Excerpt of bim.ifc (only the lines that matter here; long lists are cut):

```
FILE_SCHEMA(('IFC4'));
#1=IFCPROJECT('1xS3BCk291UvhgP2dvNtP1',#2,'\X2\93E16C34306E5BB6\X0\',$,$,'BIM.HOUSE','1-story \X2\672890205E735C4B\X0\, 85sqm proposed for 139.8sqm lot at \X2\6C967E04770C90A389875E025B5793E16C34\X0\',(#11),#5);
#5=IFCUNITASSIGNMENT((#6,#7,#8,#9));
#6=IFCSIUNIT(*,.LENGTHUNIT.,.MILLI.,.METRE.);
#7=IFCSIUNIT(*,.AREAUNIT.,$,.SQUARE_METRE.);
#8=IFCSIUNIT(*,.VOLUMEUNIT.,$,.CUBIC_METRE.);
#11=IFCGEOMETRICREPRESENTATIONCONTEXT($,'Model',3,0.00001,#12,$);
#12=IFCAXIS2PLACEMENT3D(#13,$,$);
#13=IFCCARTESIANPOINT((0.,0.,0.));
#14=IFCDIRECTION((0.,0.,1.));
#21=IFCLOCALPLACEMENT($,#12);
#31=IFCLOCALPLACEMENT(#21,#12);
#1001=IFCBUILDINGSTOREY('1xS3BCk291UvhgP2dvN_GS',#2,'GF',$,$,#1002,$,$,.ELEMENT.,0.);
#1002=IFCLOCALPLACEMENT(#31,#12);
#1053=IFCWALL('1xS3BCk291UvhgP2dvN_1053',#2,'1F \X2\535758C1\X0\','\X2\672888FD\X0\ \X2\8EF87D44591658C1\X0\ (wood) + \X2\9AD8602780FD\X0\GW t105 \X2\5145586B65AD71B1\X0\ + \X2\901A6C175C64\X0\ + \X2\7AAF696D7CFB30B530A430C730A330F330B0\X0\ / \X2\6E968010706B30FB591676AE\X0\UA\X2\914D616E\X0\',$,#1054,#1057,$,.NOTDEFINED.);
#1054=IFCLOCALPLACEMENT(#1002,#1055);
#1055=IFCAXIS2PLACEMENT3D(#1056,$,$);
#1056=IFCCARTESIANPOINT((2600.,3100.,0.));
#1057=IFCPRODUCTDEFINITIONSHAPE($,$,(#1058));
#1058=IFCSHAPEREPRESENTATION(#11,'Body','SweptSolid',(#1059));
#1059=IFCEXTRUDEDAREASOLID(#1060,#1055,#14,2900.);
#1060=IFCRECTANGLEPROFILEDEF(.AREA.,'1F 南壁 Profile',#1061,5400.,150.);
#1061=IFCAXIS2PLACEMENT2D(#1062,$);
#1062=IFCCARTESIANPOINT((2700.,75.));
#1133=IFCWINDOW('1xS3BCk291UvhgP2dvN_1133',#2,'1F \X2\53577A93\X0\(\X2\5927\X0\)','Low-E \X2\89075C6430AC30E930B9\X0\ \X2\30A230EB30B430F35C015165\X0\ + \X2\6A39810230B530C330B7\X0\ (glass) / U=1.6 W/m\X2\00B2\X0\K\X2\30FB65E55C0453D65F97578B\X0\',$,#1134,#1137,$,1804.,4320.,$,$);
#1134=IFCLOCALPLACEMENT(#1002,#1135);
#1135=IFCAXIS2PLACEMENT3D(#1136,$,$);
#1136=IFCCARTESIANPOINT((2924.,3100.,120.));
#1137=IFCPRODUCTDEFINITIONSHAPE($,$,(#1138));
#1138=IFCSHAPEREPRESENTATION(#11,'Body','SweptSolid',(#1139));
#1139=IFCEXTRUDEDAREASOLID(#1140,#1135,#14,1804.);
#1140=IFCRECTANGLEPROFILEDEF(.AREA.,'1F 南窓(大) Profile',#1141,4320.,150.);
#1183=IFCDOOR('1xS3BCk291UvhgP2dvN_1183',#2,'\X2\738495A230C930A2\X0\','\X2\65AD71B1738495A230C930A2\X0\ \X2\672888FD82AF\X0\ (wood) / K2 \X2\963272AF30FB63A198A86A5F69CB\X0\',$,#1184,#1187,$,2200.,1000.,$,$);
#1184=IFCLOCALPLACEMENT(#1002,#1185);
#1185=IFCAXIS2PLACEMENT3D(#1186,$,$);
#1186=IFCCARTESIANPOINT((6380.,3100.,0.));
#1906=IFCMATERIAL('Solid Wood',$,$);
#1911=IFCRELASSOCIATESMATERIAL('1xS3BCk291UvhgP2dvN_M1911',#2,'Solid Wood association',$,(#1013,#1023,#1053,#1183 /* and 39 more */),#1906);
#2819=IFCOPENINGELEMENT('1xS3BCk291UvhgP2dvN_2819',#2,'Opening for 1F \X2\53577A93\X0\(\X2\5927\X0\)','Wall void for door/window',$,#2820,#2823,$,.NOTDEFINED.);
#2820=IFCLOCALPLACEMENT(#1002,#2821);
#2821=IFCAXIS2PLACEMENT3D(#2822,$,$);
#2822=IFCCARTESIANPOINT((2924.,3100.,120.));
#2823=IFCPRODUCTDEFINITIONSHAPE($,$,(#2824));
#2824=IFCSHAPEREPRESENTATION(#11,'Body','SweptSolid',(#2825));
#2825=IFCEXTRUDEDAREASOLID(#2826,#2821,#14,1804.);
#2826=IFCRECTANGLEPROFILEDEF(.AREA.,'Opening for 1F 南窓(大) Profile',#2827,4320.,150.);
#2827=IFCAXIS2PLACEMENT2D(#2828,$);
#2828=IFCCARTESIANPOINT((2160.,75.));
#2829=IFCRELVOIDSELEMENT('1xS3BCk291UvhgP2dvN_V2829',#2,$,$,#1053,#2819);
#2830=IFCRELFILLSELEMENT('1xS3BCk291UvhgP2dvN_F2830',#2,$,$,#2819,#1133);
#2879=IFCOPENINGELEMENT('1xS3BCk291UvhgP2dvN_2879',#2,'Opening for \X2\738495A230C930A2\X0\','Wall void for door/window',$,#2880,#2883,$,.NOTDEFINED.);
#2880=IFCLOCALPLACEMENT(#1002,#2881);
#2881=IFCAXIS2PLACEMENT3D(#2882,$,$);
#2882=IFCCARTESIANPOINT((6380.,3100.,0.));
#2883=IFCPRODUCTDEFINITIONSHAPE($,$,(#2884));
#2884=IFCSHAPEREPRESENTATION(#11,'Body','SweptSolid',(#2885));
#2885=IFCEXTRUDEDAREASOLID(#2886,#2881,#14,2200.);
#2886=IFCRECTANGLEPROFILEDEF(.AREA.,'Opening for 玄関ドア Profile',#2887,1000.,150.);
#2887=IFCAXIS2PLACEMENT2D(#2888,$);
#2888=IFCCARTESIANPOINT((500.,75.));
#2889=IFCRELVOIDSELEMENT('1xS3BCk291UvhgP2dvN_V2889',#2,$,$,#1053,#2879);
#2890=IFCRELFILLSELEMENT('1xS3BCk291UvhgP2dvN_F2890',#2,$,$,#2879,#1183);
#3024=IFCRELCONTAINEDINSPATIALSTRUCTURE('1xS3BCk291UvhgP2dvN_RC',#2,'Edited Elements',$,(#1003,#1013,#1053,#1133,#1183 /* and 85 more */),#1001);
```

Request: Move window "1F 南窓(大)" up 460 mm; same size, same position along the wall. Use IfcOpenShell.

```python
import numpy as np
import ifcopenshell
import ifcopenshell.api.geometry
import ifcopenshell.util.placement
import ifcopenshell.util.unit

model = ifcopenshell.open("bim.ifc")
unit_scale = ifcopenshell.util.unit.calculate_unit_scale(model)

window = model.by_guid("1xS3BCk291UvhgP2dvN_1133")
opening = window.FillsVoids[0].RelatingOpeningElement
dz = 0.46 / unit_scale

shift = np.array([0.0, 0.0, dz])
# The window is not placed relative to its opening, so move both.
for product in (opening, window):
    matrix = ifcopenshell.util.placement.get_local_placement(product.ObjectPlacement)
    matrix[:3, 3] += shift
    ifcopenshell.api.geometry.edit_object_placement(model, product=product, matrix=matrix, is_si=False)

print(f"moved by {dz * unit_scale:+.3f} m")

model.write("bim_v2.ifc")
```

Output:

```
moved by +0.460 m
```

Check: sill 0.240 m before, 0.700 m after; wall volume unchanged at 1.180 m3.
